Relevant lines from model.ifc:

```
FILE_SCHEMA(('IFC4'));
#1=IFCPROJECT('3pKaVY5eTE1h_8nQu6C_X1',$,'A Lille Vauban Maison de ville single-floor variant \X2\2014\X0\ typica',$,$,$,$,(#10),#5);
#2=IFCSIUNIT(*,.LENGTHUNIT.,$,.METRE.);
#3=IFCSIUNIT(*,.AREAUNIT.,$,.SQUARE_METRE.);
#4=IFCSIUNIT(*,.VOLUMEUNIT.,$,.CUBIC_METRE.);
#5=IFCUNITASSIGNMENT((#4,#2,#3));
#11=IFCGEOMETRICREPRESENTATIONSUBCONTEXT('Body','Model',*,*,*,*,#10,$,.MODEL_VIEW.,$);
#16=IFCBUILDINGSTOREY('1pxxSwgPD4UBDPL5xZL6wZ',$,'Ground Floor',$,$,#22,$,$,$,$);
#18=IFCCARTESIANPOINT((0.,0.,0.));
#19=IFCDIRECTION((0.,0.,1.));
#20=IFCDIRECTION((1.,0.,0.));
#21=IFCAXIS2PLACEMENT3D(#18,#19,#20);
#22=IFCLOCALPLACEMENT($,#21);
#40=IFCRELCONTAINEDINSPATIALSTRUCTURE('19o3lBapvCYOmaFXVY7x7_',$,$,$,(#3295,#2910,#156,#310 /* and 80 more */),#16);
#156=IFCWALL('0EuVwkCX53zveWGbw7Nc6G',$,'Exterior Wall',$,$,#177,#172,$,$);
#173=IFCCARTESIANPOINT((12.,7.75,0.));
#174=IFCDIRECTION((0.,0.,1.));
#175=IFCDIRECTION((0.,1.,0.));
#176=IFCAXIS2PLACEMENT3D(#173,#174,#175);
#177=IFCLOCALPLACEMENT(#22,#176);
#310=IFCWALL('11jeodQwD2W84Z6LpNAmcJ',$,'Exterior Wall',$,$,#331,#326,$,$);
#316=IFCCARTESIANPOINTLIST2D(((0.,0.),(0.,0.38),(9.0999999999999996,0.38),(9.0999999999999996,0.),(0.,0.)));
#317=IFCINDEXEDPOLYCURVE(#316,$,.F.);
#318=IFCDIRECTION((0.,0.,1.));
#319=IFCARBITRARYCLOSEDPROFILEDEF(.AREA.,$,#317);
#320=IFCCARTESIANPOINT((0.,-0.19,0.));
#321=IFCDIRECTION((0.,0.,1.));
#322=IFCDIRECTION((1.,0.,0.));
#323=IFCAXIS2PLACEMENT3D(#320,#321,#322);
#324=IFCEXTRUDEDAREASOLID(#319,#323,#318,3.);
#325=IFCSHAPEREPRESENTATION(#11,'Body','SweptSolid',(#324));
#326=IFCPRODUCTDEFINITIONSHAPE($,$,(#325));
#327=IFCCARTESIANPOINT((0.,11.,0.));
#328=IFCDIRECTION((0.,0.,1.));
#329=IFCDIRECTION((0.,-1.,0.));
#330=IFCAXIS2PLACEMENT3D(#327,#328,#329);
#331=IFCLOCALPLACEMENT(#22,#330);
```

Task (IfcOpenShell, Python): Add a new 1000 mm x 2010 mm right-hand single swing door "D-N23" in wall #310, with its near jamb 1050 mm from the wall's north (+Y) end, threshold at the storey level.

```python
import numpy as np
import ifcopenshell
import ifcopenshell.api.feature
import ifcopenshell.api.geometry
import ifcopenshell.api.root
import ifcopenshell.api.spatial
import ifcopenshell.geom
import ifcopenshell.util.element
import ifcopenshell.util.placement
import ifcopenshell.util.representation
import ifcopenshell.util.shape
import ifcopenshell.util.unit

model = ifcopenshell.open("model.ifc")
unit_scale = ifcopenshell.util.unit.calculate_unit_scale(model)
settings = ifcopenshell.geom.settings()


def volume(element):
    """Net volume in cubic metres, openings subtracted."""
    shape = ifcopenshell.geom.create_shape(settings, element)
    return ifcopenshell.util.shape.get_volume(shape.geometry)


wall = model.by_guid("11jeodQwD2W84Z6LpNAmcJ")
storey = ifcopenshell.util.element.get_container(wall, ifc_class="IfcBuildingStorey")
context = ifcopenshell.util.representation.get_context(model, "Model", "Body", "MODEL_VIEW")
before = volume(wall)

width, height, from_end, sill = 1, 2.01, 1.05, 0.0  # metres

# The wall runs along its own X axis, and the end named is its -X end.
wall_shape = ifcopenshell.geom.create_shape(settings, wall)
x, y, z = ifcopenshell.util.shape.get_vertices(wall_shape.geometry).T
start = x.min() + from_end
face, thickness = float(y.min()), float(y.max() - y.min())
wall_matrix = ifcopenshell.util.placement.get_local_placement(wall.ObjectPlacement)
level = ifcopenshell.util.placement.get_local_placement(storey.ObjectPlacement)[2, 3]


def in_wall(x, y):
    """Placement at x, y metres in the wall's axes, at sill height."""
    matrix = wall_matrix.copy()
    matrix[:, 3] = wall_matrix @ np.array([x / unit_scale, y / unit_scale, 0.0, 1.0])
    matrix[2, 3] = level + sill / unit_scale
    return matrix


# Opening: a box that overshoots both wall faces by 50 mm.
opening = ifcopenshell.api.root.create_entity(model, ifc_class="IfcOpeningElement", predefined_type="OPENING")
box = ifcopenshell.api.geometry.add_wall_representation(
    model, context=context, length=width, height=height, thickness=thickness + 0.1
)
ifcopenshell.api.geometry.assign_representation(model, product=opening, representation=box)
ifcopenshell.api.geometry.edit_object_placement(model, product=opening, matrix=in_wall(start, face - 0.05), is_si=False)
ifcopenshell.api.feature.add_feature(model, feature=opening, element=wall)

door = ifcopenshell.api.root.create_entity(model, ifc_class="IfcDoor", name="D-N23", predefined_type="DOOR")
door.OverallWidth, door.OverallHeight = width / unit_scale, height / unit_scale
door.OperationType = "SINGLE_SWING_RIGHT"
body = ifcopenshell.api.geometry.add_door_representation(
    model,
    context=context,
    overall_width=door.OverallWidth,
    overall_height=door.OverallHeight,
    operation_type="SINGLE_SWING_RIGHT",
    lining_properties={"LiningDepth": thickness / unit_scale, "ThresholdDepth": thickness / unit_scale},
)
ifcopenshell.api.geometry.assign_representation(model, product=door, representation=body)
ifcopenshell.api.spatial.assign_container(model, products=[door], relating_structure=storey)
ifcopenshell.api.feature.add_filling(model, opening=opening, element=door)

# The lining spans the wall, so the door starts at the wall face.
ifcopenshell.api.geometry.edit_object_placement(model, product=door, matrix=in_wall(start, face), is_si=False)

after = volume(wall)

print(f"wall volume {before:.3f} -> {after:.3f} m3")

model.write("model_v2.ifc")
```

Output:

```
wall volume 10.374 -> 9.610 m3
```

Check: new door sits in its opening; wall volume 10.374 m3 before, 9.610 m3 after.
